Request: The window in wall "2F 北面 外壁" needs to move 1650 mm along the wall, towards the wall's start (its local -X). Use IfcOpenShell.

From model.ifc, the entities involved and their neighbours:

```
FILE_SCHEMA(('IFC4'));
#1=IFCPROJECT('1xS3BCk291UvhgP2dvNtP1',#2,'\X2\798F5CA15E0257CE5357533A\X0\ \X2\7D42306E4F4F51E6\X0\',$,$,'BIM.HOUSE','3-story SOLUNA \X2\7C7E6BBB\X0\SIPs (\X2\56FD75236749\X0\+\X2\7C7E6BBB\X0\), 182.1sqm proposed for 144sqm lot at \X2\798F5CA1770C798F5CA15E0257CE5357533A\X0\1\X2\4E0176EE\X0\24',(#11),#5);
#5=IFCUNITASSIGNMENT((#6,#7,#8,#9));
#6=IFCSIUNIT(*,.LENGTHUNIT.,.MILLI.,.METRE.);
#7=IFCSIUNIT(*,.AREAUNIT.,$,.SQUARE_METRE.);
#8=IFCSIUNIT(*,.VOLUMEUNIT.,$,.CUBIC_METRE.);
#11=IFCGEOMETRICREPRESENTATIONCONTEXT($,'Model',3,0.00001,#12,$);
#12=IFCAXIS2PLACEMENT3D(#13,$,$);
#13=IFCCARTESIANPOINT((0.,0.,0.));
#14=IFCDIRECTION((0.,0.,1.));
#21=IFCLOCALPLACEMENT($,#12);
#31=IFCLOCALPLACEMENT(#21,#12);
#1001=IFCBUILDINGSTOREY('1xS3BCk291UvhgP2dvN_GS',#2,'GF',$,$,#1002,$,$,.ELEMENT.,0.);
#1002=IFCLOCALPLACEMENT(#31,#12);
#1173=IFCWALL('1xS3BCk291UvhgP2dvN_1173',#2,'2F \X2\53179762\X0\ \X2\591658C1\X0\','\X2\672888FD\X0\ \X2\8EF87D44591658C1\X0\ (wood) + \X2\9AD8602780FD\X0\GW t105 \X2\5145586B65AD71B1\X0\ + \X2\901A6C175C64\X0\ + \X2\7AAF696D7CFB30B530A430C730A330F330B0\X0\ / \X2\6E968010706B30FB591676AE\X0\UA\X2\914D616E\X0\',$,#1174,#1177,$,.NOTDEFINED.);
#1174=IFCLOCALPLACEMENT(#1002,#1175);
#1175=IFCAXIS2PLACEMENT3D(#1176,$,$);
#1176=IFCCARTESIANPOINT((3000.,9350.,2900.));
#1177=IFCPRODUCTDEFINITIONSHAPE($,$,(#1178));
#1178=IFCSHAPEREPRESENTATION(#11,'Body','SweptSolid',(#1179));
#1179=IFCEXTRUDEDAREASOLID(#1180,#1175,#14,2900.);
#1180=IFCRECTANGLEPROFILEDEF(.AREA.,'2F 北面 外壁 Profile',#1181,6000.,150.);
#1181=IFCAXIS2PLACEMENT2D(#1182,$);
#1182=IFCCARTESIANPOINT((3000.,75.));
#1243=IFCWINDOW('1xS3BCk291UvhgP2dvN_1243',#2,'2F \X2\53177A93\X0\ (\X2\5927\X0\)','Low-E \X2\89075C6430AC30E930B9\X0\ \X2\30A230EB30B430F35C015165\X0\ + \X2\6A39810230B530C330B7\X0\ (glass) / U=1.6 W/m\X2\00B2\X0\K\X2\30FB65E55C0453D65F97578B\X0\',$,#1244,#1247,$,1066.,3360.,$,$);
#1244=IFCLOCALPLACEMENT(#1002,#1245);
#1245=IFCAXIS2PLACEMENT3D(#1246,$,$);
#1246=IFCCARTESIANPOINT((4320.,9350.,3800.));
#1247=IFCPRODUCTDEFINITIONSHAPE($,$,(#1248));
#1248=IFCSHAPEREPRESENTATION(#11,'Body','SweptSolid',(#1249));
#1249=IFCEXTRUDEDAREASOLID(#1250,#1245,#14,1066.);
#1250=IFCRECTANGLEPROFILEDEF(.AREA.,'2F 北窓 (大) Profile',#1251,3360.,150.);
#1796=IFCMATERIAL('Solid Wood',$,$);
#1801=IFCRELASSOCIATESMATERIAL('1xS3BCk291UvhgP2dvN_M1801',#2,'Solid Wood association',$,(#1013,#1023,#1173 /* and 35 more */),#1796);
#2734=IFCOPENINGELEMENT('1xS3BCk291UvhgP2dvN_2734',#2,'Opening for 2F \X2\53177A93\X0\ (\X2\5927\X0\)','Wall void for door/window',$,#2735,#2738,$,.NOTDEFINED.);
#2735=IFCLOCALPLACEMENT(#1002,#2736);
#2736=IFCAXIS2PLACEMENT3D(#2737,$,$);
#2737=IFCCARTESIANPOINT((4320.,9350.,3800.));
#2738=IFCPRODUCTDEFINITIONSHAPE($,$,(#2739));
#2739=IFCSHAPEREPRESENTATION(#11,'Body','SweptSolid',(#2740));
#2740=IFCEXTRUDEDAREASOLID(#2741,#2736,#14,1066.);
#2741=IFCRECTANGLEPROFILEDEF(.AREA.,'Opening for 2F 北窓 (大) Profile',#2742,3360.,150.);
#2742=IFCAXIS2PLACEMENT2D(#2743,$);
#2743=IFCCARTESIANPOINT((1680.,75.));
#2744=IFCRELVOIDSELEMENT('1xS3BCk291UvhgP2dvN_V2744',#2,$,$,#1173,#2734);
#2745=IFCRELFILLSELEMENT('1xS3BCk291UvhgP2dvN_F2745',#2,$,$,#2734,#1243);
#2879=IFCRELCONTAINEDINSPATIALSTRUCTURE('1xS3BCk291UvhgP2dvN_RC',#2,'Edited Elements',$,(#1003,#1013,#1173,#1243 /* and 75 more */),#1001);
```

```python
import ifcopenshell
import ifcopenshell.api.geometry
import ifcopenshell.util.placement
import ifcopenshell.util.unit

model = ifcopenshell.open("model.ifc")
unit_scale = ifcopenshell.util.unit.calculate_unit_scale(model)

window = model.by_guid("1xS3BCk291UvhgP2dvN_1243")
opening = window.FillsVoids[0].RelatingOpeningElement
wall = opening.VoidsElements[0].RelatingBuildingElement

wall_matrix = ifcopenshell.util.placement.get_local_placement(wall.ObjectPlacement)
shift = wall_matrix[:3, 0] * -1.65 / unit_scale
before = ifcopenshell.util.placement.get_local_placement(window.ObjectPlacement)[:3, 3].copy()

# The window is not placed relative to its opening, so move both.
for product in (opening, window):
    matrix = ifcopenshell.util.placement.get_local_placement(product.ObjectPlacement)
    matrix[:3, 3] += shift
    ifcopenshell.api.geometry.edit_object_placement(model, product=product, matrix=matrix, is_si=False)

after = ifcopenshell.util.placement.get_local_placement(window.ObjectPlacement)[:3, 3]
print("window moved by", (after - before).round(3) + 0.0)

model.write("model-out.ifc")
```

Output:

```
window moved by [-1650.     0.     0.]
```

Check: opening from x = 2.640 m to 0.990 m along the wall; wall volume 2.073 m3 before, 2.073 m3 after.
